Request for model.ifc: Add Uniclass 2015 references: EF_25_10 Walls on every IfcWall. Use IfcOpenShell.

First a look at what the model holds.

```python
import ifcopenshell

model = ifcopenshell.open("model.ifc")
print(model.schema)
print("classifications:", [c.Name for c in model.by_type("IfcClassification")])
for ifc_class in ("IfcDoor", "IfcRoof", "IfcStair", "IfcWall", "IfcWindow"):
    print(ifc_class, len(model.by_type(ifc_class)))
```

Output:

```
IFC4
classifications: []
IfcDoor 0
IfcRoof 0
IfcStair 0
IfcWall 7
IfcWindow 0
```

```python
import ifcopenshell
import ifcopenshell.api.classification

model = ifcopenshell.open("model.ifc")

system = ifcopenshell.api.classification.add_classification(model, classification="Uniclass 2015")

codes = {
    "IfcWall": ("EF_25_10", "Walls"),
}
for ifc_class, (code, name) in codes.items():
    products = model.by_type(ifc_class)
    ifcopenshell.api.classification.add_reference(
        model, products=products, classification=system, identification=code, name=name
    )
    print(code, len(products))

model.write("model_updated.ifc")
```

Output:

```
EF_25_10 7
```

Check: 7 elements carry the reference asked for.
